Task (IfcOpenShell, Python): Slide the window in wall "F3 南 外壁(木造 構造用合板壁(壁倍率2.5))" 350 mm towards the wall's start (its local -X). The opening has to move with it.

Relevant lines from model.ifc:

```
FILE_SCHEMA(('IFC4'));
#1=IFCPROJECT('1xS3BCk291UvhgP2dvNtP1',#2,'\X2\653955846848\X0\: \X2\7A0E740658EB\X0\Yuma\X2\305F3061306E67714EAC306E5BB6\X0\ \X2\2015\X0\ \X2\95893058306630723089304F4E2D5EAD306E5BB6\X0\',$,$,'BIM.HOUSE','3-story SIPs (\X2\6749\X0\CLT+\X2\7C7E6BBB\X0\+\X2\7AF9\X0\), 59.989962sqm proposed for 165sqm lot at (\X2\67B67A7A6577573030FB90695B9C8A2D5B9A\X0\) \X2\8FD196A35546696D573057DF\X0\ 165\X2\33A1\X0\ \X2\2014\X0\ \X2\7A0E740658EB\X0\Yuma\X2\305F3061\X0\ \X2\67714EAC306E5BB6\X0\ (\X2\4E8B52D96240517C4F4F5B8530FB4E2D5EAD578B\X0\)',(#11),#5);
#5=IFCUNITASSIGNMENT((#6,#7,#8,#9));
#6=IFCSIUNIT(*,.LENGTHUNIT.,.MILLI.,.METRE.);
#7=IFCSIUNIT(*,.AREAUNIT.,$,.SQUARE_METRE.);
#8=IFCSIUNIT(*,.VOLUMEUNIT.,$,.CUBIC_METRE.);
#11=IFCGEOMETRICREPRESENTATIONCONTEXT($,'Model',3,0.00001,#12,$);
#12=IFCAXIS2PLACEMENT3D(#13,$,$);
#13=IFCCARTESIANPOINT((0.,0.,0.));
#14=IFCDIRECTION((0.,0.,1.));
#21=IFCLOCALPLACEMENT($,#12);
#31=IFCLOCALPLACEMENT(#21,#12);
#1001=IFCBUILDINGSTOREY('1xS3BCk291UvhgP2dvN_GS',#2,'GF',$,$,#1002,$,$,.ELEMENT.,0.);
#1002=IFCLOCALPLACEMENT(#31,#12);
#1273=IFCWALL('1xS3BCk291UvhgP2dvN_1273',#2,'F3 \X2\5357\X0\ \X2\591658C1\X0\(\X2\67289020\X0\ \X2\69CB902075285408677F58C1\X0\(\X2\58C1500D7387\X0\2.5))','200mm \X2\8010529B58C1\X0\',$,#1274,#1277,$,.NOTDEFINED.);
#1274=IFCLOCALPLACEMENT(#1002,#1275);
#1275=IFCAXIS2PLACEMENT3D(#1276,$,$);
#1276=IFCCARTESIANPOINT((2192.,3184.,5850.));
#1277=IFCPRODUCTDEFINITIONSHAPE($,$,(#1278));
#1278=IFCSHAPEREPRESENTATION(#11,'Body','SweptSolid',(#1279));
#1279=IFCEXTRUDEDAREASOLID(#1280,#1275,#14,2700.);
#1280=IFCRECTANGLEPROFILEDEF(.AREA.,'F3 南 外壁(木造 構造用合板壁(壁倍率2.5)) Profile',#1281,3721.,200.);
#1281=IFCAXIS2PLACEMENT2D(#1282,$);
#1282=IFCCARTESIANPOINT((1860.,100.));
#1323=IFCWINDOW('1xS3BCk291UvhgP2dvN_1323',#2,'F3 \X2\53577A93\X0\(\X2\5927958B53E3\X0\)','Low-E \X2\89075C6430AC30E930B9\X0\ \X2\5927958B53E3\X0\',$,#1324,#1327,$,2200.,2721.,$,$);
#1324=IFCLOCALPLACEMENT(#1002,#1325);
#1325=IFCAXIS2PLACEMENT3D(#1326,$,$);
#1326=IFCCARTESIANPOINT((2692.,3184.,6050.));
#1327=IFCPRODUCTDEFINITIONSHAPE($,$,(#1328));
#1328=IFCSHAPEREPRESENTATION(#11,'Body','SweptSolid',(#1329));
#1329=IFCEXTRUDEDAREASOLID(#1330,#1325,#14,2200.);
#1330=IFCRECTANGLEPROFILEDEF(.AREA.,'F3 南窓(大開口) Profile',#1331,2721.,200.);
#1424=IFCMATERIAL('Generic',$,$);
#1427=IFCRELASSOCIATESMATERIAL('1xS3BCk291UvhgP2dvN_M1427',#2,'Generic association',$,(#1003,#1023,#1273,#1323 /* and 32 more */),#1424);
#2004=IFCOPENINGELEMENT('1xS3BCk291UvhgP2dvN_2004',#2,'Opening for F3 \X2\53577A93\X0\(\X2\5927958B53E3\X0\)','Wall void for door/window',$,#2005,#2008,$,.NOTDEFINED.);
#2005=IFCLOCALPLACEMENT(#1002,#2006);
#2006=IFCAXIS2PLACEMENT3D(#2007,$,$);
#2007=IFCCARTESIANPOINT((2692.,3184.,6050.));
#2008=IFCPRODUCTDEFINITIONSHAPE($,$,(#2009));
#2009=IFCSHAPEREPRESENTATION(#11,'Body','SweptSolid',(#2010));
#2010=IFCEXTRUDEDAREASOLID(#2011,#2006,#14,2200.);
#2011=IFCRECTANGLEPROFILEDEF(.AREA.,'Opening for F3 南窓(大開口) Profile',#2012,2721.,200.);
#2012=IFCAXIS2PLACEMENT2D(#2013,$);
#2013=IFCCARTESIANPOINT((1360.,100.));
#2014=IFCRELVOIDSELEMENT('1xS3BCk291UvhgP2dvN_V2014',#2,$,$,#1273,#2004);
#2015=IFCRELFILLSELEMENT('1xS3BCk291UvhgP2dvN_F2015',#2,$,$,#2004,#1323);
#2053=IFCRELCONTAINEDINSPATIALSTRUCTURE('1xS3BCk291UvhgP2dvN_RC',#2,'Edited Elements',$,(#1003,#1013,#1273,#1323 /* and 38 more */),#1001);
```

```python
import ifcopenshell
import ifcopenshell.api.geometry
import ifcopenshell.util.placement

model = ifcopenshell.open("model.ifc")

window = model.by_guid("1xS3BCk291UvhgP2dvN_1323")
opening = window.FillsVoids[0].RelatingOpeningElement
wall = opening.VoidsElements[0].RelatingBuildingElement

wall_matrix = ifcopenshell.util.placement.get_local_placement(wall.ObjectPlacement)
shift = wall_matrix[:3, 0] * -350.0
before = ifcopenshell.util.placement.get_local_placement(window.ObjectPlacement)[:3, 3].copy()

# The window is not placed relative to its opening, so move both.
for product in (opening, window):
    matrix = ifcopenshell.util.placement.get_local_placement(product.ObjectPlacement)
    matrix[:3, 3] += shift
    ifcopenshell.api.geometry.edit_object_placement(model, product=product, matrix=matrix, is_si=False)

after = ifcopenshell.util.placement.get_local_placement(window.ObjectPlacement)[:3, 3]
print("window moved by", (after - before).round(3) + 0.0)

model.write("model_edited.ifc")
```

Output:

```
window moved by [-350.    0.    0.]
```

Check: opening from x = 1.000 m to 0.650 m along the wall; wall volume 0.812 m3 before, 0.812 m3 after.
